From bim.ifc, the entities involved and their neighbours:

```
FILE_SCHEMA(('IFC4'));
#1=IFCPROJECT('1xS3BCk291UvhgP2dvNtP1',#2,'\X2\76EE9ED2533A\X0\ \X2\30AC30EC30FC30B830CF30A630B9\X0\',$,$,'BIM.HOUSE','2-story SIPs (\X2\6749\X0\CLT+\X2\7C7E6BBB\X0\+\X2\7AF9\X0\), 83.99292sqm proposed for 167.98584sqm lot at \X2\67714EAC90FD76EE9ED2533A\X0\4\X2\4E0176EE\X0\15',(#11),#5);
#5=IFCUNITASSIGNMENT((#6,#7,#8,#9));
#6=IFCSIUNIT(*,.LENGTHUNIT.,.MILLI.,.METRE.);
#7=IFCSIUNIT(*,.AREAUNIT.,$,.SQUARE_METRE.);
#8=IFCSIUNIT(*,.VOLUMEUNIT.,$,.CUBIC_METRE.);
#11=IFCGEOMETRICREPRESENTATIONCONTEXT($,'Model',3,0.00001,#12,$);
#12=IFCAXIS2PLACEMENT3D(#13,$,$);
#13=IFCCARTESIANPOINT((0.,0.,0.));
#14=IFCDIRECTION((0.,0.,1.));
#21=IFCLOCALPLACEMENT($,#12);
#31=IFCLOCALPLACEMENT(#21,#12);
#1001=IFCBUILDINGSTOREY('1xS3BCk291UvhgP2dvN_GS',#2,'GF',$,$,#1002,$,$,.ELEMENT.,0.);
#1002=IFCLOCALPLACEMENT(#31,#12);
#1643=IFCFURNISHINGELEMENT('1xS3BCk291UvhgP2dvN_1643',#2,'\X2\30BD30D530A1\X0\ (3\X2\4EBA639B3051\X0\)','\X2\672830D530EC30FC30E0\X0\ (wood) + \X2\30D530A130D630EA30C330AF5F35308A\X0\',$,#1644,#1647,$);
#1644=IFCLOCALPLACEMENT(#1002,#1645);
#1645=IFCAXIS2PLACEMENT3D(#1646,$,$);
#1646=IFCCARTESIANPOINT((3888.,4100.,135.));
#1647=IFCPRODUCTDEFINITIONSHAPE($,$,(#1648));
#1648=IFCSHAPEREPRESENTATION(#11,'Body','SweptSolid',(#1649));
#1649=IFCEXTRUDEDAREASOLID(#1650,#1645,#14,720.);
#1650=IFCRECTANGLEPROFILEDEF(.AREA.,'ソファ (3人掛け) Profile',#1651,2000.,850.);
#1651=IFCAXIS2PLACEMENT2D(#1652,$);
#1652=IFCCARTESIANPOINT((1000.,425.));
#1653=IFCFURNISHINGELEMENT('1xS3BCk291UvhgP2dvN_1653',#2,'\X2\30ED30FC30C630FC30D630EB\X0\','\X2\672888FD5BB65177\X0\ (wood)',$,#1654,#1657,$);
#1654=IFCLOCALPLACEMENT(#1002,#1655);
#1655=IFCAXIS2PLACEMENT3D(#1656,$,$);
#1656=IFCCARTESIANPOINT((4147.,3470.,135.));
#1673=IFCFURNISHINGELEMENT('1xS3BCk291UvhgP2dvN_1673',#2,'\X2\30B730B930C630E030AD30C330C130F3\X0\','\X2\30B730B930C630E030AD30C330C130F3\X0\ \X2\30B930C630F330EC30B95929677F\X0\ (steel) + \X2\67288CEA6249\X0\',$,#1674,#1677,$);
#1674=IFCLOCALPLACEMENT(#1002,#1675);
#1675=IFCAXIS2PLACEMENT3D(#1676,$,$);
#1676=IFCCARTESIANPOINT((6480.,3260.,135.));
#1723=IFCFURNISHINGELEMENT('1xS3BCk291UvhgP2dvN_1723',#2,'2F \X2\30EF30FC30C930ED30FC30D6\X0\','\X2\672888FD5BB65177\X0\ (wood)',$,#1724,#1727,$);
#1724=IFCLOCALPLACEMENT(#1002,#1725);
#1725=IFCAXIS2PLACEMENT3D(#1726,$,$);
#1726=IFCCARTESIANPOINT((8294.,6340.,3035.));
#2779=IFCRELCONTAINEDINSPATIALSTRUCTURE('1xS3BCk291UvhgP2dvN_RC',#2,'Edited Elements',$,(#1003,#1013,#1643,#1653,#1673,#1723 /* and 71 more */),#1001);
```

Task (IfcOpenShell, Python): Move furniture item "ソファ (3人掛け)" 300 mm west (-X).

```python
import ifcopenshell
import ifcopenshell.api.geometry
import ifcopenshell.util.placement
import ifcopenshell.util.unit

model = ifcopenshell.open("bim.ifc")
unit_scale = ifcopenshell.util.unit.calculate_unit_scale(model)

item = model.by_guid("1xS3BCk291UvhgP2dvN_1643")
matrix = ifcopenshell.util.placement.get_local_placement(item.ObjectPlacement)
matrix[0, 3] -= 0.3 / unit_scale
ifcopenshell.api.geometry.edit_object_placement(model, product=item, matrix=matrix, is_si=False)

print(ifcopenshell.util.placement.get_local_placement(item.ObjectPlacement).round(3) + 0.0)

model.write("bim_rev.ifc")
```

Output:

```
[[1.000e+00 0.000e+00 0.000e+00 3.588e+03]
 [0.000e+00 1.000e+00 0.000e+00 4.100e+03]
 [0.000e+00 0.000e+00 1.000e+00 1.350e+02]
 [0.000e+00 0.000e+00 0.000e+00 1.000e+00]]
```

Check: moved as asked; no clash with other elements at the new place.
